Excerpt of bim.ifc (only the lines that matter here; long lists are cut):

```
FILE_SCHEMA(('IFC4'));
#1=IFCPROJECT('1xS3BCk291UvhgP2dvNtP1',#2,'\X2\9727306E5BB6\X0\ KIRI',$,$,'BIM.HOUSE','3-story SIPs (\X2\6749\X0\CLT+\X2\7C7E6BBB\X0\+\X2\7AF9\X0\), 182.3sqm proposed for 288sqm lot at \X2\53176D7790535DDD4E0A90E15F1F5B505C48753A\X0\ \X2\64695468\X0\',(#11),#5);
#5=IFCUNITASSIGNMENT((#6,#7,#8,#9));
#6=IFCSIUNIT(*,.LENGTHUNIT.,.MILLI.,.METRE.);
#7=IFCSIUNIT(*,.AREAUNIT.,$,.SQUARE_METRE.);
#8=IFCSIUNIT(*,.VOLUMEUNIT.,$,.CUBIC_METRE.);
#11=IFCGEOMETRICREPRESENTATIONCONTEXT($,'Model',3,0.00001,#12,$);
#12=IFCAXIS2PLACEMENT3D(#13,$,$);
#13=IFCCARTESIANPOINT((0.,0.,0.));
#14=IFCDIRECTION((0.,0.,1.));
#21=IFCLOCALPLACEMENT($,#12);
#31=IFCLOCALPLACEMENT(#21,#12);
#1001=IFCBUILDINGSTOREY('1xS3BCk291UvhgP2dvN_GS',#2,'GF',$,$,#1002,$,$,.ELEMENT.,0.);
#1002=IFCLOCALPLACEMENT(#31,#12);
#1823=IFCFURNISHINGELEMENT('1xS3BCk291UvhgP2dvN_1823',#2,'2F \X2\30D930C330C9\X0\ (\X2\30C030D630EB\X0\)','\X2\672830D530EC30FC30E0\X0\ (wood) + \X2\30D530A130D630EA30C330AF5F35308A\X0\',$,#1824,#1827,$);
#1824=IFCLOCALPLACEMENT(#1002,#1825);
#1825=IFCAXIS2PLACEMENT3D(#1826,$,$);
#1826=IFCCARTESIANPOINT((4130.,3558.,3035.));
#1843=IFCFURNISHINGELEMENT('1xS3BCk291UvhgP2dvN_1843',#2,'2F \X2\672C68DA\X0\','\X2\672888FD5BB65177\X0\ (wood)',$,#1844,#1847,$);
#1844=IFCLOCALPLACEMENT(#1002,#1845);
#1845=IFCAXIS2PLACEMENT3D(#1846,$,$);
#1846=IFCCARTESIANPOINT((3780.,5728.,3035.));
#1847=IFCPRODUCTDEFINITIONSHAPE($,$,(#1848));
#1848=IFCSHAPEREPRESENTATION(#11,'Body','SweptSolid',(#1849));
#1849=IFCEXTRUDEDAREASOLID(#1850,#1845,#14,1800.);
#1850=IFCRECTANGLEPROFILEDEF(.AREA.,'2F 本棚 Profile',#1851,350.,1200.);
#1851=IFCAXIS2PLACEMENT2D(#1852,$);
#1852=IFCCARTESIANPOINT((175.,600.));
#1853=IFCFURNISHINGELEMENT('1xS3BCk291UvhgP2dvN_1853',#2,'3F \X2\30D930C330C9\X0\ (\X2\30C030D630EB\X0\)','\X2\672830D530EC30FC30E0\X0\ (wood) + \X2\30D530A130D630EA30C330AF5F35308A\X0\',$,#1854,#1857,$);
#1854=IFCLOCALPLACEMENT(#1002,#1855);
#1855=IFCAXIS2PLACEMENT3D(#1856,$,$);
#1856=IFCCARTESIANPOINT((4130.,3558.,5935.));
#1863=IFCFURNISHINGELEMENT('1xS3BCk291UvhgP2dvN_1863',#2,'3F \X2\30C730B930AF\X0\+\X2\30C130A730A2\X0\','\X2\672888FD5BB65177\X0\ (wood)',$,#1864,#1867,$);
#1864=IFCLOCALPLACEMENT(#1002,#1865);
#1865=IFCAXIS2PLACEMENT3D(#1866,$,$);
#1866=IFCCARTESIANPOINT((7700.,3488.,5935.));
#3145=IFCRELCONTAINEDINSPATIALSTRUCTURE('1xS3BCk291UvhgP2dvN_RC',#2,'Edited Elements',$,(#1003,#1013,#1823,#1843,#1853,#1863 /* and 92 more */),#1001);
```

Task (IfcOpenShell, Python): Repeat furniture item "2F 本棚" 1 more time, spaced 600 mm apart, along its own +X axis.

```python
import ifcopenshell
import ifcopenshell.api.geometry
import ifcopenshell.api.root
import ifcopenshell.util.element
import ifcopenshell.util.placement
import ifcopenshell.util.unit

model = ifcopenshell.open("bim.ifc")
unit_scale = ifcopenshell.util.unit.calculate_unit_scale(model)


def reuse_history(source, copy):
    """copy_class also copies each property set's owner history, people and application; keep the originals."""
    for rel in copy.IsDefinedBy:
        if rel.is_a("IfcRelDefinesByProperties") and (history := rel.RelatingPropertyDefinition.OwnerHistory):
            rel.RelatingPropertyDefinition.OwnerHistory = source.OwnerHistory
            ifcopenshell.util.element.remove_deep2(model, history)


source = model.by_guid("1xS3BCk291UvhgP2dvN_1843")
base = ifcopenshell.util.placement.get_local_placement(source.ObjectPlacement)
step = base[:3, 0] * 0.6 / unit_scale

for i in range(1, 2):
    copy = ifcopenshell.api.root.copy_class(model, product=source)
    copy.Representation = ifcopenshell.util.element.copy_deep(
        model, source.Representation, exclude=["IfcGeometricRepresentationContext", "IfcRepresentationMap"]
    )
    reuse_history(source, copy)
    matrix = base.copy()
    matrix[:3, 3] += i * step
    print("added at", matrix[:3, 3].round(3) + 0.0)
    ifcopenshell.api.geometry.edit_object_placement(model, product=copy, matrix=matrix, is_si=False)

model.write("bim_rev.ifc")
```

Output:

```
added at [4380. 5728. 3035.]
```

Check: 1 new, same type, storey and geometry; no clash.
